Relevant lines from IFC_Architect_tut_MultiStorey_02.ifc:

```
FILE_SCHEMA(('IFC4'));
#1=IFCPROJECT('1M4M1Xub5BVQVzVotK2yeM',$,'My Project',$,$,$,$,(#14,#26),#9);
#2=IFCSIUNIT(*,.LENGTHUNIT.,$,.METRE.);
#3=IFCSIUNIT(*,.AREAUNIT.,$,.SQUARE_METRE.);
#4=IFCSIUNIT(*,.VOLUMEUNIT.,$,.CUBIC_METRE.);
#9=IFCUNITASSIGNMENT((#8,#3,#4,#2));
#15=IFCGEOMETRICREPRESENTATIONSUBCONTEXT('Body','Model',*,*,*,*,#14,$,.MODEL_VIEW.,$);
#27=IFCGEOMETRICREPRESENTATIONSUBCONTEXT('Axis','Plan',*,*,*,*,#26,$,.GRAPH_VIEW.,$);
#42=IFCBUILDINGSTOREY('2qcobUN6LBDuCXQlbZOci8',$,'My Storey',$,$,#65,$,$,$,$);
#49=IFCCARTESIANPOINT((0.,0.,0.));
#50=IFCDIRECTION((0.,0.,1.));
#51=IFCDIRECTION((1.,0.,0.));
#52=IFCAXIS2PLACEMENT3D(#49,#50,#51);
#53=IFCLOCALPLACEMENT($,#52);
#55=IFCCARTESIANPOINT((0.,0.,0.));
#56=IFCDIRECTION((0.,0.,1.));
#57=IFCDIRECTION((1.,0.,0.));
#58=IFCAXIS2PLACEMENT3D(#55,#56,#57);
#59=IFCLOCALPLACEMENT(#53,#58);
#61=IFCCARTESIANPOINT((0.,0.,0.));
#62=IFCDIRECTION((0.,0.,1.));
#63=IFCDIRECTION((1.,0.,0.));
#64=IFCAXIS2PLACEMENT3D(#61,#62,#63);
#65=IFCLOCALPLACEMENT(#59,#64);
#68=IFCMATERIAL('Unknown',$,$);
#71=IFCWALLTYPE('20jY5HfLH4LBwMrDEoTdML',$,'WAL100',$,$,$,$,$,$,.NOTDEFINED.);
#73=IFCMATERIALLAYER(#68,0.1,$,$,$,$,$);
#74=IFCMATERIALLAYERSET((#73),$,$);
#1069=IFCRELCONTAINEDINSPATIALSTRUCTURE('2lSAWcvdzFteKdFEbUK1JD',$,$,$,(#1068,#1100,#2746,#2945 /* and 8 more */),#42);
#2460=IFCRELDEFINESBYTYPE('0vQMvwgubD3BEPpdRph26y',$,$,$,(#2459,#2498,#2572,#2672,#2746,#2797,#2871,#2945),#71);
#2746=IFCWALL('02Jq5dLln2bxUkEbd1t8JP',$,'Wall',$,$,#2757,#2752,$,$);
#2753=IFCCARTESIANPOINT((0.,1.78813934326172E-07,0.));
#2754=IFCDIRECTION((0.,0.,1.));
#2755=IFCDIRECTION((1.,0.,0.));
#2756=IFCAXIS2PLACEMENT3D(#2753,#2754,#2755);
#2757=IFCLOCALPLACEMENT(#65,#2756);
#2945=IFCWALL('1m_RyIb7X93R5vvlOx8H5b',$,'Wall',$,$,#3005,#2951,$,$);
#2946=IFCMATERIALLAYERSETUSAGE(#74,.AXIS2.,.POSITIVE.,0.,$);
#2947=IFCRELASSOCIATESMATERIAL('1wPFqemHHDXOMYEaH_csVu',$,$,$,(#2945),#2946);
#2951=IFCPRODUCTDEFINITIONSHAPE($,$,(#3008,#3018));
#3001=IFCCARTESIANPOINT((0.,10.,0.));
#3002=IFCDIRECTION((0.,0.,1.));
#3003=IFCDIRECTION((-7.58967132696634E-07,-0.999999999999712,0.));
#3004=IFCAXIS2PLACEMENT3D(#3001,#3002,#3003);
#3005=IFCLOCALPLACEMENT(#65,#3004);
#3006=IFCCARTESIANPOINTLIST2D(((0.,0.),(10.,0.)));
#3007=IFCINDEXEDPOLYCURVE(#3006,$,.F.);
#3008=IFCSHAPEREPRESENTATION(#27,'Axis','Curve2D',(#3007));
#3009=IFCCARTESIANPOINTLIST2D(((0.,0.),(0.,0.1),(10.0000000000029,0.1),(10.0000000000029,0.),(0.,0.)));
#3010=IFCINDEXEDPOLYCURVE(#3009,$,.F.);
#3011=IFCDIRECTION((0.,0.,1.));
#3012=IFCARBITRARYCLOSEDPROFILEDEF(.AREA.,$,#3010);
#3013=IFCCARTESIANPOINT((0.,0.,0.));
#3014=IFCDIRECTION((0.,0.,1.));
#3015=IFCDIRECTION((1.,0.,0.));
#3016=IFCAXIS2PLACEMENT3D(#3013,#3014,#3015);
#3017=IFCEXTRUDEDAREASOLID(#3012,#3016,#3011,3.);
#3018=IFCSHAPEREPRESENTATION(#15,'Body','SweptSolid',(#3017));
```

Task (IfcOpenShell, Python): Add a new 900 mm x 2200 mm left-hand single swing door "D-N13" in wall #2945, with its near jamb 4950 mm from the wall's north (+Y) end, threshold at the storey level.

```python
import numpy as np
import ifcopenshell
import ifcopenshell.api.feature
import ifcopenshell.api.geometry
import ifcopenshell.api.root
import ifcopenshell.api.spatial
import ifcopenshell.geom
import ifcopenshell.util.element
import ifcopenshell.util.placement
import ifcopenshell.util.representation
import ifcopenshell.util.shape
import ifcopenshell.util.unit

model = ifcopenshell.open("IFC_Architect_tut_MultiStorey_02.ifc")
unit_scale = ifcopenshell.util.unit.calculate_unit_scale(model)
settings = ifcopenshell.geom.settings()


def volume(element):
    """Net volume in cubic metres, openings subtracted."""
    shape = ifcopenshell.geom.create_shape(settings, element)
    return ifcopenshell.util.shape.get_volume(shape.geometry)


wall = model.by_guid("1m_RyIb7X93R5vvlOx8H5b")
storey = ifcopenshell.util.element.get_container(wall, ifc_class="IfcBuildingStorey")
context = ifcopenshell.util.representation.get_context(model, "Model", "Body", "MODEL_VIEW")
before = volume(wall)

width, height, from_end, sill = 0.9, 2.2, 4.95, 0.0  # metres

# The wall runs along its own X axis, and the end named is its -X end.
wall_shape = ifcopenshell.geom.create_shape(settings, wall)
x, y, z = ifcopenshell.util.shape.get_vertices(wall_shape.geometry).T
start = x.min() + from_end
face, thickness = float(y.min()), float(y.max() - y.min())
wall_matrix = ifcopenshell.util.placement.get_local_placement(wall.ObjectPlacement)
level = ifcopenshell.util.placement.get_local_placement(storey.ObjectPlacement)[2, 3]


def in_wall(x, y):
    """Placement at x, y metres in the wall's axes, at sill height."""
    matrix = wall_matrix.copy()
    matrix[:, 3] = wall_matrix @ np.array([x / unit_scale, y / unit_scale, 0.0, 1.0])
    matrix[2, 3] = level + sill / unit_scale
    return matrix


# Opening: a box that overshoots both wall faces by 50 mm.
opening = ifcopenshell.api.root.create_entity(model, ifc_class="IfcOpeningElement", predefined_type="OPENING")
box = ifcopenshell.api.geometry.add_wall_representation(
    model, context=context, length=width, height=height, thickness=thickness + 0.1
)
ifcopenshell.api.geometry.assign_representation(model, product=opening, representation=box)
ifcopenshell.api.geometry.edit_object_placement(model, product=opening, matrix=in_wall(start, face - 0.05), is_si=False)
ifcopenshell.api.feature.add_feature(model, feature=opening, element=wall)

door = ifcopenshell.api.root.create_entity(model, ifc_class="IfcDoor", name="D-N13", predefined_type="DOOR")
door.OverallWidth, door.OverallHeight = width / unit_scale, height / unit_scale
door.OperationType = "SINGLE_SWING_LEFT"
body = ifcopenshell.api.geometry.add_door_representation(
    model,
    context=context,
    overall_width=door.OverallWidth,
    overall_height=door.OverallHeight,
    operation_type="SINGLE_SWING_LEFT",
    lining_properties={"LiningDepth": thickness / unit_scale, "ThresholdDepth": thickness / unit_scale},
)
ifcopenshell.api.geometry.assign_representation(model, product=door, representation=body)
ifcopenshell.api.spatial.assign_container(model, products=[door], relating_structure=storey)
ifcopenshell.api.feature.add_filling(model, opening=opening, element=door)

# The lining spans the wall, so the door starts at the wall face.
ifcopenshell.api.geometry.edit_object_placement(model, product=door, matrix=in_wall(start, face), is_si=False)

after = volume(wall)

print(f"wall volume {before:.3f} -> {after:.3f} m3")

model.write("IFC_Architect_tut_MultiStorey_02_edited.ifc")
```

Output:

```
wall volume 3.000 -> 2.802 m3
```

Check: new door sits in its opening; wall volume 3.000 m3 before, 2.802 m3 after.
